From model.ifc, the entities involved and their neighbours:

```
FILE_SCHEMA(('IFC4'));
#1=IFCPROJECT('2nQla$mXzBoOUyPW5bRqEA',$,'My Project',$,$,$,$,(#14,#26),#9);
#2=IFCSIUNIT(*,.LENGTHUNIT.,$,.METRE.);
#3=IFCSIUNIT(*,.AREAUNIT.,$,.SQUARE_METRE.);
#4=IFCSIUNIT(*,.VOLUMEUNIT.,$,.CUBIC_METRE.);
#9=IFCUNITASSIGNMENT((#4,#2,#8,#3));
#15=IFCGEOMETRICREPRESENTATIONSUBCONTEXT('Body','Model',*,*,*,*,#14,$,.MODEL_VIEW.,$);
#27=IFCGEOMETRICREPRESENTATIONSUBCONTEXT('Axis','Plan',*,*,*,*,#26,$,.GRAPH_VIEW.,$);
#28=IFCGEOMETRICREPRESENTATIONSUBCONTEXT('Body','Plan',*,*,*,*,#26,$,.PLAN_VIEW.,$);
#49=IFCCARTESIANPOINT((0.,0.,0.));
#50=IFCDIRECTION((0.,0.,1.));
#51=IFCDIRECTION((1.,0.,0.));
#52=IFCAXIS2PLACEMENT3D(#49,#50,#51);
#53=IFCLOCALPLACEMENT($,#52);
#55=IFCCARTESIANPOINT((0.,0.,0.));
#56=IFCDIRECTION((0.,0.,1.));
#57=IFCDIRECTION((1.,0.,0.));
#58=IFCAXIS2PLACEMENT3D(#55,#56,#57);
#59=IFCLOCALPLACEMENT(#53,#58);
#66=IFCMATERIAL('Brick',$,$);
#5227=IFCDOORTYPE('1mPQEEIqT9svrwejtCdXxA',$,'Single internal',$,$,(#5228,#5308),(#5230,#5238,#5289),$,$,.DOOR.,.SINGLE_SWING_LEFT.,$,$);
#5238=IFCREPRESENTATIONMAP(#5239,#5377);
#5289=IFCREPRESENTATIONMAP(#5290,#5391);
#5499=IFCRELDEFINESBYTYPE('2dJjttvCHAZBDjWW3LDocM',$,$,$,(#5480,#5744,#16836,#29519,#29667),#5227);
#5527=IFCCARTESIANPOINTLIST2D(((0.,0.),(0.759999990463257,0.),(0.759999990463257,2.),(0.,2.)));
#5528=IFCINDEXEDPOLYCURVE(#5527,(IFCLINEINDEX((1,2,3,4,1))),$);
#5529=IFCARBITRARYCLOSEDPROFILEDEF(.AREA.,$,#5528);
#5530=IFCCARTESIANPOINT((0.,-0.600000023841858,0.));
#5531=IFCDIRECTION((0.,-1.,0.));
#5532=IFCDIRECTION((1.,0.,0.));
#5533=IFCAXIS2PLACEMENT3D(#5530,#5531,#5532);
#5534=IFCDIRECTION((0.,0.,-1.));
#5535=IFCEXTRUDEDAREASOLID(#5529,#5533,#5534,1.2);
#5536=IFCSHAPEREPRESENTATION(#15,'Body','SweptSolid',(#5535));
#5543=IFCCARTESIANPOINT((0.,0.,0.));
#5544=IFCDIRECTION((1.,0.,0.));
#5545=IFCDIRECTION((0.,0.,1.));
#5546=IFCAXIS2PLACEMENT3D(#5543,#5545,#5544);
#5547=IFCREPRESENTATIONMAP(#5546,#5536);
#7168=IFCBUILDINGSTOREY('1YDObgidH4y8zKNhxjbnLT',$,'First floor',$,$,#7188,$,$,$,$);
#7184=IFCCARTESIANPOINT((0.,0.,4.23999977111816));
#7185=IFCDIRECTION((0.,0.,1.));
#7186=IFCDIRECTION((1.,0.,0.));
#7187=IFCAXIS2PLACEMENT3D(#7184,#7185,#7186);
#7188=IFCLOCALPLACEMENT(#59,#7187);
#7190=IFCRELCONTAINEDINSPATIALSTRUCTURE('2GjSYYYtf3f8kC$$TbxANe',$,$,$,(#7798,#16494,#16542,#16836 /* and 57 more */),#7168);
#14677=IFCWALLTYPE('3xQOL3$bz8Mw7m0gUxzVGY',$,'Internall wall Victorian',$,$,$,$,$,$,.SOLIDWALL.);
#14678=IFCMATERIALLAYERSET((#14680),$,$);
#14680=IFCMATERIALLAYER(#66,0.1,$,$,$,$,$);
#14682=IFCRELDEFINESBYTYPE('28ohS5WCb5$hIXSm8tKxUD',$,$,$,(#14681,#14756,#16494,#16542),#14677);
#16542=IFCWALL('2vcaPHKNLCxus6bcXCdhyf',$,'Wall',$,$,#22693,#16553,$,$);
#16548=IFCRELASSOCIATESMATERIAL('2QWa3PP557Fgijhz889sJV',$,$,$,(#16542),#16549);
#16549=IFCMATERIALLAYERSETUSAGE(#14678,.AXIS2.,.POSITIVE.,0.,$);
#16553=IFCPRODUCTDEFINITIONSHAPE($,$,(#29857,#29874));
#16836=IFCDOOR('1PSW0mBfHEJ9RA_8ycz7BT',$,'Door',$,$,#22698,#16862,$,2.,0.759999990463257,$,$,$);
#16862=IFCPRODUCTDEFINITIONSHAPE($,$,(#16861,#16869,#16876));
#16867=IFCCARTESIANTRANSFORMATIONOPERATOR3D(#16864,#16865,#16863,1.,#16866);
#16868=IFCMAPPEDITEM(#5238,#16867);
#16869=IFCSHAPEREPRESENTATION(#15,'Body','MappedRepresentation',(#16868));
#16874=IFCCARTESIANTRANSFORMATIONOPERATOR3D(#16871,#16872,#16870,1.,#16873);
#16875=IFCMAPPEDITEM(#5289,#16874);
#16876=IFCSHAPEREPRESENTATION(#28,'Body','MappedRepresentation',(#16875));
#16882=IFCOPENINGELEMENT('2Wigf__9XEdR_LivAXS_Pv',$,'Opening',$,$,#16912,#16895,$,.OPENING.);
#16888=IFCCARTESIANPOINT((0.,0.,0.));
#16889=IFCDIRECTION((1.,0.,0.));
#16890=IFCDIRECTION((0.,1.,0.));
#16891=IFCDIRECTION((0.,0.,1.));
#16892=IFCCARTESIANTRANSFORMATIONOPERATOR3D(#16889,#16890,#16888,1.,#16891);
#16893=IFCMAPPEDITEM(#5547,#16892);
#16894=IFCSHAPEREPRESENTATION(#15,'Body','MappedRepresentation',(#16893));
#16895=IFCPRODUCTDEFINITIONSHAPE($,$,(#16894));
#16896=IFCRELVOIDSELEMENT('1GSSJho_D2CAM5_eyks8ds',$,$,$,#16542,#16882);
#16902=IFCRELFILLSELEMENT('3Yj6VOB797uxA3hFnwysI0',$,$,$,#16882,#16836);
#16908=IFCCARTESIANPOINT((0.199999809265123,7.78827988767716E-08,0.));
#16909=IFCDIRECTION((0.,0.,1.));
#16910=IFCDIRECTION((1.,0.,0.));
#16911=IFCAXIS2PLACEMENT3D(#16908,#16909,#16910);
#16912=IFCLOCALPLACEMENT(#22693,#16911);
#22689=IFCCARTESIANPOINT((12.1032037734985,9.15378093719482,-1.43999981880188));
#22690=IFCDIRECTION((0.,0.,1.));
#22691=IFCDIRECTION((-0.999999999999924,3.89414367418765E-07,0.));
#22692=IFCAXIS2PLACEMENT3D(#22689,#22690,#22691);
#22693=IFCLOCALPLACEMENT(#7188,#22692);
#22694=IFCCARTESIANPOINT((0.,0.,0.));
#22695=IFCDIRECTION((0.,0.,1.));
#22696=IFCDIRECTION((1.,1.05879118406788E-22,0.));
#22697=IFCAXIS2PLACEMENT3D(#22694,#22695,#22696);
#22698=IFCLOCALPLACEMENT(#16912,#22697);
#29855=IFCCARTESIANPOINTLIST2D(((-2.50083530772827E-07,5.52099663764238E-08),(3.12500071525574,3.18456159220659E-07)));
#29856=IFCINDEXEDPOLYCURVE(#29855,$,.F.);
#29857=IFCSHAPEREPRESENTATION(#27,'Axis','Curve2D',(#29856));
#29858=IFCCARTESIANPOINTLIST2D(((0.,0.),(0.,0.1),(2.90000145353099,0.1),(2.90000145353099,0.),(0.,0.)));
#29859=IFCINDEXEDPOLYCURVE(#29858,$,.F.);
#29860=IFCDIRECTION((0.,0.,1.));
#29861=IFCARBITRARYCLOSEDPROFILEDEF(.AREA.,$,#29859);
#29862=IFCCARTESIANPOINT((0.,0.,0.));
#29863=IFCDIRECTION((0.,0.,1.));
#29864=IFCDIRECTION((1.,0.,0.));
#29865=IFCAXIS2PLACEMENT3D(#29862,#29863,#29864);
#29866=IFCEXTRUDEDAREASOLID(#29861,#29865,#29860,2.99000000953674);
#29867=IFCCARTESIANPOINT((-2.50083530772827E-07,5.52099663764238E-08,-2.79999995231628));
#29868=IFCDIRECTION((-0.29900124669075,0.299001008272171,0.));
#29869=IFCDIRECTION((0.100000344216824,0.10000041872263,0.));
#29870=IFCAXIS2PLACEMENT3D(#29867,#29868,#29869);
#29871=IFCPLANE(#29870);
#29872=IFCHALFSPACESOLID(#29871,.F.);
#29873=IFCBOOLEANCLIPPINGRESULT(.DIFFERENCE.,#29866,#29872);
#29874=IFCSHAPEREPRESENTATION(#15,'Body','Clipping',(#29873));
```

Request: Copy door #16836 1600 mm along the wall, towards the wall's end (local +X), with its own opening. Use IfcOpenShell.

```python
import ifcopenshell
import ifcopenshell.api.feature
import ifcopenshell.api.geometry
import ifcopenshell.api.root
import ifcopenshell.geom
import ifcopenshell.util.element
import ifcopenshell.util.placement
import ifcopenshell.util.shape
import ifcopenshell.util.unit

model = ifcopenshell.open("model.ifc")
unit_scale = ifcopenshell.util.unit.calculate_unit_scale(model)
settings = ifcopenshell.geom.settings()


def volume(element):
    """Net volume in cubic metres, openings subtracted."""
    shape = ifcopenshell.geom.create_shape(settings, element)
    return ifcopenshell.util.shape.get_volume(shape.geometry)


door = model.by_id(16836)
opening = door.FillsVoids[0].RelatingOpeningElement
wall = opening.VoidsElements[0].RelatingBuildingElement
before = volume(wall)
shift = ifcopenshell.util.placement.get_local_placement(wall.ObjectPlacement)[:3, 0] * 1.6 / unit_scale

# copy_class copies the void relationship, type, container and properties, but no geometry.
new_opening = ifcopenshell.api.root.copy_class(model, product=opening)
new_opening.Representation = ifcopenshell.util.element.copy_deep(
    model, opening.Representation, exclude=["IfcGeometricRepresentationContext", "IfcRepresentationMap"]
)
new_door = ifcopenshell.api.root.copy_class(model, product=door)
new_door.Representation = ifcopenshell.util.element.copy_deep(
    model, door.Representation, exclude=["IfcGeometricRepresentationContext", "IfcRepresentationMap"]
)
ifcopenshell.api.feature.add_filling(model, opening=new_opening, element=new_door)

for old, new in ((opening, new_opening), (door, new_door)):
    matrix = ifcopenshell.util.placement.get_local_placement(old.ObjectPlacement)
    matrix[:3, 3] += shift
    ifcopenshell.api.geometry.edit_object_placement(model, product=new, matrix=matrix, is_si=False)

after = volume(wall)

print(f"wall volume {before:.3f} -> {after:.3f} m3")

model.write("model_edited.ifc")
```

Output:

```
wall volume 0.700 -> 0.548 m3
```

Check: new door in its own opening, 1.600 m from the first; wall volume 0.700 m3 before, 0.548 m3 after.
